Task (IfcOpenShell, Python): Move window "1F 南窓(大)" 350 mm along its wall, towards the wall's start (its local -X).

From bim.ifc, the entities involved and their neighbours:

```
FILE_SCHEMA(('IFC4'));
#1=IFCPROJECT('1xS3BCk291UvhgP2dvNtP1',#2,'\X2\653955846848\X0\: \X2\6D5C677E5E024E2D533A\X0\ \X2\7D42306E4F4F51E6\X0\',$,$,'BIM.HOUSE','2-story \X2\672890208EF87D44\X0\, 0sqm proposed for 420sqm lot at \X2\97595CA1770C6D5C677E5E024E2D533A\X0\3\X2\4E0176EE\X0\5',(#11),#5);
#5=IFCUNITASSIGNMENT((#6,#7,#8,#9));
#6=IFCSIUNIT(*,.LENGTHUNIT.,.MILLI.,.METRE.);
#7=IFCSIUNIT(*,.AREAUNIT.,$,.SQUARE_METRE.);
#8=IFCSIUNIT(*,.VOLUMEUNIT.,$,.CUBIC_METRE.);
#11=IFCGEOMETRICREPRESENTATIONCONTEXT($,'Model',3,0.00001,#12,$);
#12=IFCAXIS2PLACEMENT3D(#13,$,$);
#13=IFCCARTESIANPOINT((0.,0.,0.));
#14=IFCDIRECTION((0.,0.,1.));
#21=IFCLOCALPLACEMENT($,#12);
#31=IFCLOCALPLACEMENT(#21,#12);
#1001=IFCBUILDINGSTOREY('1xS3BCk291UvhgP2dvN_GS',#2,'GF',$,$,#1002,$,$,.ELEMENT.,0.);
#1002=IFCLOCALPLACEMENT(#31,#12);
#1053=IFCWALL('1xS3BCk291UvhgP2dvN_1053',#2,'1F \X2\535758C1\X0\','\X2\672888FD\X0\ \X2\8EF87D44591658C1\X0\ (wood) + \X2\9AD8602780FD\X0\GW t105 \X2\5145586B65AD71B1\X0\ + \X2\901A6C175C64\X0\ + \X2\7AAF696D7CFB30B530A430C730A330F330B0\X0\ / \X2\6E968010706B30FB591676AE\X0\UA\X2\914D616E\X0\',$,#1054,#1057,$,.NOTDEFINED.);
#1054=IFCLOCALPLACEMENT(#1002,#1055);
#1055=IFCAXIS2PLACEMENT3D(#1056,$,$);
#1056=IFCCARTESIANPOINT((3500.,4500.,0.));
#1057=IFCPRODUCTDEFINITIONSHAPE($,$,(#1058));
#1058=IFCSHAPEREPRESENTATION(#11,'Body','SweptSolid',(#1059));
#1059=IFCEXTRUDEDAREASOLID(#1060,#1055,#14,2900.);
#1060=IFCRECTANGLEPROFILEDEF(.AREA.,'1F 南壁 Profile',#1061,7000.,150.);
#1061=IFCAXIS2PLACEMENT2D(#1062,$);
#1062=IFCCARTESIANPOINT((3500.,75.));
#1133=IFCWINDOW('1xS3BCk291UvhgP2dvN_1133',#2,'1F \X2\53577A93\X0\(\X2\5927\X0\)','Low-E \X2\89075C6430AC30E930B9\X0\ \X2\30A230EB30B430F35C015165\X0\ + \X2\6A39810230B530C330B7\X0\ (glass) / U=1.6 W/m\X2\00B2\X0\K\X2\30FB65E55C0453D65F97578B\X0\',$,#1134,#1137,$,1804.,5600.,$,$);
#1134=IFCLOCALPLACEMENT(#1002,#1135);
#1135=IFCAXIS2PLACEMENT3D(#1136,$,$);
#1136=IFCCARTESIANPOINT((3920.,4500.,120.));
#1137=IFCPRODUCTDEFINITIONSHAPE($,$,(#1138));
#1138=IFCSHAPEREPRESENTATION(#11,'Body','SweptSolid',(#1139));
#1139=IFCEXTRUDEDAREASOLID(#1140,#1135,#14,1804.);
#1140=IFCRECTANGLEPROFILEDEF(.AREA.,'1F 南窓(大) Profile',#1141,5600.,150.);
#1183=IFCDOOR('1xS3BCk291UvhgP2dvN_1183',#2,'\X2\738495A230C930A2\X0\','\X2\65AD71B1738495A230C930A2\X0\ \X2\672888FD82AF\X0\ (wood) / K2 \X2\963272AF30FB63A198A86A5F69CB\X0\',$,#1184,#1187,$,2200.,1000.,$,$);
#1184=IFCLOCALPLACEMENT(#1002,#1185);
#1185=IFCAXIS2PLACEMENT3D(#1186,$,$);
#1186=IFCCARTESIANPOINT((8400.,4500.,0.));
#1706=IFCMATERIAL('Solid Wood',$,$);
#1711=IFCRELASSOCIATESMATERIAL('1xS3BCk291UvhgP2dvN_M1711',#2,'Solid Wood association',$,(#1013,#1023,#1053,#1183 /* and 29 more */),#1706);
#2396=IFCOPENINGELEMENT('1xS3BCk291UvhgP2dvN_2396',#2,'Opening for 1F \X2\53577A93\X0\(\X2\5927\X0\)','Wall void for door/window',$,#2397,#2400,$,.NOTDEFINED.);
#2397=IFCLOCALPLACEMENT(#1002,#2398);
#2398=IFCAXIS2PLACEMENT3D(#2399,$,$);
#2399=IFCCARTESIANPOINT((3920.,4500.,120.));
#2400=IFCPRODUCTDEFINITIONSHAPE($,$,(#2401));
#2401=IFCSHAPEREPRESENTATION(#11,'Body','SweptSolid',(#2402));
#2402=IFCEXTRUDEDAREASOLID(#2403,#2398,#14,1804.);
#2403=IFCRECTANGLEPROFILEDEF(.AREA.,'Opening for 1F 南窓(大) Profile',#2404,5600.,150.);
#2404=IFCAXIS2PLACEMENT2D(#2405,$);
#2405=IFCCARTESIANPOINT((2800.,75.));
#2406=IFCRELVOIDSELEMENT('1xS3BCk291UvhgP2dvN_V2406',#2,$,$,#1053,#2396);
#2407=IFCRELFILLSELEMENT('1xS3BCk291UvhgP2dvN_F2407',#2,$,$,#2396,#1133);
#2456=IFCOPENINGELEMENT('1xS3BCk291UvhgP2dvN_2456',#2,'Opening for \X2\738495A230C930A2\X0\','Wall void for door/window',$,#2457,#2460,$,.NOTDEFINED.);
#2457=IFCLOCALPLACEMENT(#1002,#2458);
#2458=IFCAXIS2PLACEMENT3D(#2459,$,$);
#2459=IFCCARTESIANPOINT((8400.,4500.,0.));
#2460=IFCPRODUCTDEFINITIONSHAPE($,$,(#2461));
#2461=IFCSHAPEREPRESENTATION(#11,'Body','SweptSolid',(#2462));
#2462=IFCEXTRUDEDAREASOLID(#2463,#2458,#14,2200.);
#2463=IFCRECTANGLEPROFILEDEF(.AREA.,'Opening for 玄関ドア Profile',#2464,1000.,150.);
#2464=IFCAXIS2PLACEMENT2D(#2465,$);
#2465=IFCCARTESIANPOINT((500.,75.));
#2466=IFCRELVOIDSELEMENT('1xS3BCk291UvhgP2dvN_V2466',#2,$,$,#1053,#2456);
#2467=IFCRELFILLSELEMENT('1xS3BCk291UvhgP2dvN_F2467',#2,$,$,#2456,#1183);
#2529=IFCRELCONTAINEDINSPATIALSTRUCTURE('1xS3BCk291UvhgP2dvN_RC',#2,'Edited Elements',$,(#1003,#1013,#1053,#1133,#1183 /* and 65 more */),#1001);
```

```python
import ifcopenshell
import ifcopenshell.api.geometry
import ifcopenshell.util.placement
import ifcopenshell.util.unit

model = ifcopenshell.open("bim.ifc")
unit_scale = ifcopenshell.util.unit.calculate_unit_scale(model)

window = model.by_guid("1xS3BCk291UvhgP2dvN_1133")
opening = window.FillsVoids[0].RelatingOpeningElement
wall = opening.VoidsElements[0].RelatingBuildingElement

wall_matrix = ifcopenshell.util.placement.get_local_placement(wall.ObjectPlacement)
shift = wall_matrix[:3, 0] * -0.35 / unit_scale
before = ifcopenshell.util.placement.get_local_placement(window.ObjectPlacement)[:3, 3].copy()

# The window is not placed relative to its opening, so move both.
for product in (opening, window):
    matrix = ifcopenshell.util.placement.get_local_placement(product.ObjectPlacement)
    matrix[:3, 3] += shift
    ifcopenshell.api.geometry.edit_object_placement(model, product=product, matrix=matrix, is_si=False)

after = ifcopenshell.util.placement.get_local_placement(window.ObjectPlacement)[:3, 3]
print("window moved by", (after - before).round(3) + 0.0)

model.write("bim_updated.ifc")
```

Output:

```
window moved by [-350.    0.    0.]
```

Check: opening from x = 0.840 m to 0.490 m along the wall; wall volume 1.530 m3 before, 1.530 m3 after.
